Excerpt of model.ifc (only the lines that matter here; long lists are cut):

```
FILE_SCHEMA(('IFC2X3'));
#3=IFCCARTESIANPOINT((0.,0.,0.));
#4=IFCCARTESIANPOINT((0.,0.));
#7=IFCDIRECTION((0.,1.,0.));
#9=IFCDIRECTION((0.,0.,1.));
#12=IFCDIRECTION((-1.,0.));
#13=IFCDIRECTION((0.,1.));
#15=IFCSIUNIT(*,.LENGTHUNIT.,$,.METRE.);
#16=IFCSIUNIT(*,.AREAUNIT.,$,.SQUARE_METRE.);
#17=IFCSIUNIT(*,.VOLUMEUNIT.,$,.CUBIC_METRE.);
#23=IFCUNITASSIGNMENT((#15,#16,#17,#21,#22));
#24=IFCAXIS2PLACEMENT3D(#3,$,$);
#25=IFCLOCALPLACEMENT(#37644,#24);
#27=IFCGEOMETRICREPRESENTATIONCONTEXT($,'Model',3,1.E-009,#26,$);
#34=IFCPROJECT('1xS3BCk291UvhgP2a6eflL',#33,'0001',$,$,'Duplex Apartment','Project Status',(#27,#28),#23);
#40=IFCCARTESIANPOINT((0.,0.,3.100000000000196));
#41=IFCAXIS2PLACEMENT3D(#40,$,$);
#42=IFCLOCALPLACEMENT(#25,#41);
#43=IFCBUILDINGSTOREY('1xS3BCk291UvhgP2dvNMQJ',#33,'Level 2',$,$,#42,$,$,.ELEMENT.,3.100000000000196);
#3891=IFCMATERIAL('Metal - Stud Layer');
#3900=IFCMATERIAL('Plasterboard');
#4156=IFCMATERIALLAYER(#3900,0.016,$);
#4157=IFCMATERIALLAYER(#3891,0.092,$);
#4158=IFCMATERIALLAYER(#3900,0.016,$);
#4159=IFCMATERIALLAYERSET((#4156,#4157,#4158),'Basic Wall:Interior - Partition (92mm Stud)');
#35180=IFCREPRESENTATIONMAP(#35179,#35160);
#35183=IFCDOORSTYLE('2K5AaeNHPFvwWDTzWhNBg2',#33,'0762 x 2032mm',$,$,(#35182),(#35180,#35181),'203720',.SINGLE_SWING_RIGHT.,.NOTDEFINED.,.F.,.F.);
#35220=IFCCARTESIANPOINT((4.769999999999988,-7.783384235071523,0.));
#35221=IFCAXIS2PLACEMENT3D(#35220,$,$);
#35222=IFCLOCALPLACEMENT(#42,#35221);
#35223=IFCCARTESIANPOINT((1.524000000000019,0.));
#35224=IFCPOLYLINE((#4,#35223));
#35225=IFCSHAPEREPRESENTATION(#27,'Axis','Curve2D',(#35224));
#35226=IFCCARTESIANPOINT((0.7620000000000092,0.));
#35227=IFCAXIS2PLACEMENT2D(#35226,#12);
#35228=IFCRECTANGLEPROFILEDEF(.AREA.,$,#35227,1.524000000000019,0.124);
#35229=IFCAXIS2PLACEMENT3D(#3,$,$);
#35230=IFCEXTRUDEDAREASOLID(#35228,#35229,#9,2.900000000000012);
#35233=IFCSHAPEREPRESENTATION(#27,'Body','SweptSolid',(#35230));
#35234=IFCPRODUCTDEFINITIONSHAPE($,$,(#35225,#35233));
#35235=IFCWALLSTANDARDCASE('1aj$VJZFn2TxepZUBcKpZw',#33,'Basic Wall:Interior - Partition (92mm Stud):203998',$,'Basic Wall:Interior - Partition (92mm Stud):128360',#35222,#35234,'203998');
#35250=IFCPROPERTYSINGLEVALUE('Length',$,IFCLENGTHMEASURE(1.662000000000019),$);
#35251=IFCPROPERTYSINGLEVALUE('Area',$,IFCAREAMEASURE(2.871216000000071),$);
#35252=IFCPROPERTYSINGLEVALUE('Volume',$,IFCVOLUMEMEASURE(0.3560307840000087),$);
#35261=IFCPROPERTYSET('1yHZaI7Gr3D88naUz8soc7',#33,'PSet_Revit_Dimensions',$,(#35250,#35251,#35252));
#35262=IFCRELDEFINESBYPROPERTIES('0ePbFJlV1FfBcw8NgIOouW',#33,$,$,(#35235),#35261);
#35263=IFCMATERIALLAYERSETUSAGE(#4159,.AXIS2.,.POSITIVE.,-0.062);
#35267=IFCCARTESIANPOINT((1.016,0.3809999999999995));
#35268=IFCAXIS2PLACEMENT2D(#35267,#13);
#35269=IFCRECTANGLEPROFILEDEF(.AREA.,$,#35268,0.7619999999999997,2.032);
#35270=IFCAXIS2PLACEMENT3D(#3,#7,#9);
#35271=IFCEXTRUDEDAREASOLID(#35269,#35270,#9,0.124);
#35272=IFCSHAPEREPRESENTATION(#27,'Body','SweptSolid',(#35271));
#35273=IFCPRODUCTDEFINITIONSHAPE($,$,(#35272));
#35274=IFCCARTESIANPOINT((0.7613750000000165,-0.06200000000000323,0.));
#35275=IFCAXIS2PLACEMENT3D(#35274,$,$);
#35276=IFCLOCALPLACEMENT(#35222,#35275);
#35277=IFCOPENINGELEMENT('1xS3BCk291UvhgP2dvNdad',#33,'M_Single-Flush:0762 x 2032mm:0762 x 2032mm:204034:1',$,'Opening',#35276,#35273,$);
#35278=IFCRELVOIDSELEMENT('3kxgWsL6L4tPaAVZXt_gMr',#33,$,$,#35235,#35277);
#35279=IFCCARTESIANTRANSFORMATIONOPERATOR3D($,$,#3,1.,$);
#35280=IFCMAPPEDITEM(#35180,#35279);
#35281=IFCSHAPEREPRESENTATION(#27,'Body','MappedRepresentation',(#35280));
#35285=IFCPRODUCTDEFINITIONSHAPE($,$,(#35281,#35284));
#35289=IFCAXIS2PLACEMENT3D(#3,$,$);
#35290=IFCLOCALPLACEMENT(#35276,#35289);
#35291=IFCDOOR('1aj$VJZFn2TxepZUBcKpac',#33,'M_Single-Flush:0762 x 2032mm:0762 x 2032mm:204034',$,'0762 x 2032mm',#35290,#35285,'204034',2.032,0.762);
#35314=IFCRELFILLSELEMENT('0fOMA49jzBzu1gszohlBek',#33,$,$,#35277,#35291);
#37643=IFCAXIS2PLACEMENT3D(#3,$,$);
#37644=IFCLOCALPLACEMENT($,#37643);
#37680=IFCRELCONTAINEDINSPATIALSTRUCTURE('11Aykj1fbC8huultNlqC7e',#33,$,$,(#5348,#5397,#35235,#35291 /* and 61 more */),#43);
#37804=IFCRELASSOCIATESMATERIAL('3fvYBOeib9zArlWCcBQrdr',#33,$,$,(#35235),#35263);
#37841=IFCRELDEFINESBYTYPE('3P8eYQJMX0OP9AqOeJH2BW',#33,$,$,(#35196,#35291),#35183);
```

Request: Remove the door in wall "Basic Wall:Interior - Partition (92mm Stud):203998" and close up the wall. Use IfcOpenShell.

```python
import ifcopenshell
import ifcopenshell.api.feature
import ifcopenshell.api.pset
import ifcopenshell.api.root
import ifcopenshell.geom
import ifcopenshell.util.element
import ifcopenshell.util.shape
import ifcopenshell.util.unit

model = ifcopenshell.open("model.ifc")
area_scale = ifcopenshell.util.unit.calculate_unit_scale(model, "AREAUNIT")
volume_scale = ifcopenshell.util.unit.calculate_unit_scale(model, "VOLUMEUNIT")
settings = ifcopenshell.geom.settings()


def volume(element):
    """Net volume in cubic metres, openings subtracted."""
    shape = ifcopenshell.geom.create_shape(settings, element)
    return ifcopenshell.util.shape.get_volume(shape.geometry)


door = model.by_guid("1aj$VJZFn2TxepZUBcKpac")
opening = door.FillsVoids[0].RelatingOpeningElement
wall = opening.VoidsElements[0].RelatingBuildingElement
before = volume(wall)

ifcopenshell.api.root.remove_product(model, product=door)
ifcopenshell.api.feature.remove_feature(model, feature=opening)

after = volume(wall)
thickness = 0.124  # wall thickness in metres

# Update the wall's stored quantities.
pset = model.by_id(ifcopenshell.util.element.get_pset(wall, "PSet_Revit_Dimensions", should_inherit=False)["id"])
ifcopenshell.api.pset.edit_pset(model, pset=pset, properties={
    "Area": model.create_entity("IfcAreaMeasure", after / thickness / area_scale),
    "Volume": model.create_entity("IfcVolumeMeasure", after / volume_scale),
})

print(f"wall volume {before:.3f} -> {after:.3f} m3")

model.write("model-out.ifc")
```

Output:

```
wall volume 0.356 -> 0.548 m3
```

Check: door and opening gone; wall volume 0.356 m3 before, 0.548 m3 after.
